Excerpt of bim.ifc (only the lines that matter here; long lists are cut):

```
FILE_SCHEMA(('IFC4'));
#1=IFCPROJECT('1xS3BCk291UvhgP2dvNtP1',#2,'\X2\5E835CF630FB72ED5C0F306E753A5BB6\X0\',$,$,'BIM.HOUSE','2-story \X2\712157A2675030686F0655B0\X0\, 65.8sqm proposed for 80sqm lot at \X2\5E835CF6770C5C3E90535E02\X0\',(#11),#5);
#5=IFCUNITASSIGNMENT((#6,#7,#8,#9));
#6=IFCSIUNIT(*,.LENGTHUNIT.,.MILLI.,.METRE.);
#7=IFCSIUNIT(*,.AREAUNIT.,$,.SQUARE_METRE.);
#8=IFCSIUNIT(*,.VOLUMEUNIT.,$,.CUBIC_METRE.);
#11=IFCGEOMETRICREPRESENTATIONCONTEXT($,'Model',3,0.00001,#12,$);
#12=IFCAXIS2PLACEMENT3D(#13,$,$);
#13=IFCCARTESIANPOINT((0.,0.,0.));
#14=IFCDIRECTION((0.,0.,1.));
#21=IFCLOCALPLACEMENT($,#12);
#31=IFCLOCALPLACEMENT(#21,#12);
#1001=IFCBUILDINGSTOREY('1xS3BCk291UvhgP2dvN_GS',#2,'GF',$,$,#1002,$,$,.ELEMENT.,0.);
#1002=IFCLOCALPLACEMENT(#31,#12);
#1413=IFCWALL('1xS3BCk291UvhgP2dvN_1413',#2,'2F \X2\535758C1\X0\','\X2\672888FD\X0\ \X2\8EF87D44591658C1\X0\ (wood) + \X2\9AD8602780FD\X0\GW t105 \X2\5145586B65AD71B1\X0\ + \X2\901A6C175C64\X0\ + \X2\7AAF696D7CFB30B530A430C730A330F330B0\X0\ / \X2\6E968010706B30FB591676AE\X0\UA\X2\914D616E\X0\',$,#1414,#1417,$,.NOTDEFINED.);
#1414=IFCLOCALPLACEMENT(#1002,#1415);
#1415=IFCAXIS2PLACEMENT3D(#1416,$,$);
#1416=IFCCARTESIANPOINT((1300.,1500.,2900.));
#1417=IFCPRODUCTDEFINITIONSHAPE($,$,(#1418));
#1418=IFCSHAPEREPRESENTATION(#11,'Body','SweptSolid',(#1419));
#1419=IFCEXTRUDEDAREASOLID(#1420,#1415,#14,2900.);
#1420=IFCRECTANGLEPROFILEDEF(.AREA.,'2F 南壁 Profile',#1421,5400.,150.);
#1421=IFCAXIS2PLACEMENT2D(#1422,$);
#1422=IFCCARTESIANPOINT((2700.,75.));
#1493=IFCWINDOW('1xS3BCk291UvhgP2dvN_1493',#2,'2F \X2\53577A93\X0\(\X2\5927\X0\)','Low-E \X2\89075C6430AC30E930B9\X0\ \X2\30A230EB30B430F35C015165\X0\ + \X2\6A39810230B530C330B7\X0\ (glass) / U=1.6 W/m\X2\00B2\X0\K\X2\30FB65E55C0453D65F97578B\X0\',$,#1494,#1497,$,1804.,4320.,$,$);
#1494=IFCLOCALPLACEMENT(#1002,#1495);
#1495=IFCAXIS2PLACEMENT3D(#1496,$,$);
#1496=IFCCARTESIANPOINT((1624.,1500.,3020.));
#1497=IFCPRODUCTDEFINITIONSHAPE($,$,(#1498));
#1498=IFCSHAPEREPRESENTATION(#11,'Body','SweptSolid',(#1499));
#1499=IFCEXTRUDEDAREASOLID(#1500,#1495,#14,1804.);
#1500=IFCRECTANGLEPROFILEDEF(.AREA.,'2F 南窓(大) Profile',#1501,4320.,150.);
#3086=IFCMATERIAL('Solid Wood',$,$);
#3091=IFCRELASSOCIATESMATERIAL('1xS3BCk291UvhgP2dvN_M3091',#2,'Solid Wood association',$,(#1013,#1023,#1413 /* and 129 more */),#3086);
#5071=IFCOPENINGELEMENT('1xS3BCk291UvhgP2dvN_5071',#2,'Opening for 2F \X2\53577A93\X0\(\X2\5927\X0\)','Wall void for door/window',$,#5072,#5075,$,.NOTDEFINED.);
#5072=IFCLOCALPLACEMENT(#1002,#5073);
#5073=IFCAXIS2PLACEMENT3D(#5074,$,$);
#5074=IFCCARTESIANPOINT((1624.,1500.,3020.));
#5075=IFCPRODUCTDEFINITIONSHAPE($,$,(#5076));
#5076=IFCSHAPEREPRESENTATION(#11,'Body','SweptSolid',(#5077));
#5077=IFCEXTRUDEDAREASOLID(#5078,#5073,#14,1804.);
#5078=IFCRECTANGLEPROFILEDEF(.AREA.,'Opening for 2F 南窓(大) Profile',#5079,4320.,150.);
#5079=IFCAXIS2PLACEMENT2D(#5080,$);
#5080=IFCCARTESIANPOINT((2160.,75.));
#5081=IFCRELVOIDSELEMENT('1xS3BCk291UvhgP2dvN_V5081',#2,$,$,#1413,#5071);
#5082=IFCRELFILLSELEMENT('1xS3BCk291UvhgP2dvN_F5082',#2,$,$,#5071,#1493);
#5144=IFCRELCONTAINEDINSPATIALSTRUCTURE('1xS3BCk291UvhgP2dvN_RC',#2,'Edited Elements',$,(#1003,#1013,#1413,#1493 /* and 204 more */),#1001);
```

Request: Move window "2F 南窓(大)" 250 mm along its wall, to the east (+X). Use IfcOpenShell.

```python
import ifcopenshell
import ifcopenshell.api.geometry
import ifcopenshell.util.placement
import ifcopenshell.util.unit

model = ifcopenshell.open("bim.ifc")
unit_scale = ifcopenshell.util.unit.calculate_unit_scale(model)

window = model.by_id(1493)
opening = window.FillsVoids[0].RelatingOpeningElement
wall = opening.VoidsElements[0].RelatingBuildingElement

wall_matrix = ifcopenshell.util.placement.get_local_placement(wall.ObjectPlacement)
shift = wall_matrix[:3, 0] * 0.25 / unit_scale
before = ifcopenshell.util.placement.get_local_placement(window.ObjectPlacement)[:3, 3].copy()

# The window is not placed relative to its opening, so move both.
for product in (opening, window):
    matrix = ifcopenshell.util.placement.get_local_placement(product.ObjectPlacement)
    matrix[:3, 3] += shift
    ifcopenshell.api.geometry.edit_object_placement(model, product=product, matrix=matrix, is_si=False)

after = ifcopenshell.util.placement.get_local_placement(window.ObjectPlacement)[:3, 3]
print("window moved by", (after - before).round(3) + 0.0)

model.write("bim_updated.ifc")
```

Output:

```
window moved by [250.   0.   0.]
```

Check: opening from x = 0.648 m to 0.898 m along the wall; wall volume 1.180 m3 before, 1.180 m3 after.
